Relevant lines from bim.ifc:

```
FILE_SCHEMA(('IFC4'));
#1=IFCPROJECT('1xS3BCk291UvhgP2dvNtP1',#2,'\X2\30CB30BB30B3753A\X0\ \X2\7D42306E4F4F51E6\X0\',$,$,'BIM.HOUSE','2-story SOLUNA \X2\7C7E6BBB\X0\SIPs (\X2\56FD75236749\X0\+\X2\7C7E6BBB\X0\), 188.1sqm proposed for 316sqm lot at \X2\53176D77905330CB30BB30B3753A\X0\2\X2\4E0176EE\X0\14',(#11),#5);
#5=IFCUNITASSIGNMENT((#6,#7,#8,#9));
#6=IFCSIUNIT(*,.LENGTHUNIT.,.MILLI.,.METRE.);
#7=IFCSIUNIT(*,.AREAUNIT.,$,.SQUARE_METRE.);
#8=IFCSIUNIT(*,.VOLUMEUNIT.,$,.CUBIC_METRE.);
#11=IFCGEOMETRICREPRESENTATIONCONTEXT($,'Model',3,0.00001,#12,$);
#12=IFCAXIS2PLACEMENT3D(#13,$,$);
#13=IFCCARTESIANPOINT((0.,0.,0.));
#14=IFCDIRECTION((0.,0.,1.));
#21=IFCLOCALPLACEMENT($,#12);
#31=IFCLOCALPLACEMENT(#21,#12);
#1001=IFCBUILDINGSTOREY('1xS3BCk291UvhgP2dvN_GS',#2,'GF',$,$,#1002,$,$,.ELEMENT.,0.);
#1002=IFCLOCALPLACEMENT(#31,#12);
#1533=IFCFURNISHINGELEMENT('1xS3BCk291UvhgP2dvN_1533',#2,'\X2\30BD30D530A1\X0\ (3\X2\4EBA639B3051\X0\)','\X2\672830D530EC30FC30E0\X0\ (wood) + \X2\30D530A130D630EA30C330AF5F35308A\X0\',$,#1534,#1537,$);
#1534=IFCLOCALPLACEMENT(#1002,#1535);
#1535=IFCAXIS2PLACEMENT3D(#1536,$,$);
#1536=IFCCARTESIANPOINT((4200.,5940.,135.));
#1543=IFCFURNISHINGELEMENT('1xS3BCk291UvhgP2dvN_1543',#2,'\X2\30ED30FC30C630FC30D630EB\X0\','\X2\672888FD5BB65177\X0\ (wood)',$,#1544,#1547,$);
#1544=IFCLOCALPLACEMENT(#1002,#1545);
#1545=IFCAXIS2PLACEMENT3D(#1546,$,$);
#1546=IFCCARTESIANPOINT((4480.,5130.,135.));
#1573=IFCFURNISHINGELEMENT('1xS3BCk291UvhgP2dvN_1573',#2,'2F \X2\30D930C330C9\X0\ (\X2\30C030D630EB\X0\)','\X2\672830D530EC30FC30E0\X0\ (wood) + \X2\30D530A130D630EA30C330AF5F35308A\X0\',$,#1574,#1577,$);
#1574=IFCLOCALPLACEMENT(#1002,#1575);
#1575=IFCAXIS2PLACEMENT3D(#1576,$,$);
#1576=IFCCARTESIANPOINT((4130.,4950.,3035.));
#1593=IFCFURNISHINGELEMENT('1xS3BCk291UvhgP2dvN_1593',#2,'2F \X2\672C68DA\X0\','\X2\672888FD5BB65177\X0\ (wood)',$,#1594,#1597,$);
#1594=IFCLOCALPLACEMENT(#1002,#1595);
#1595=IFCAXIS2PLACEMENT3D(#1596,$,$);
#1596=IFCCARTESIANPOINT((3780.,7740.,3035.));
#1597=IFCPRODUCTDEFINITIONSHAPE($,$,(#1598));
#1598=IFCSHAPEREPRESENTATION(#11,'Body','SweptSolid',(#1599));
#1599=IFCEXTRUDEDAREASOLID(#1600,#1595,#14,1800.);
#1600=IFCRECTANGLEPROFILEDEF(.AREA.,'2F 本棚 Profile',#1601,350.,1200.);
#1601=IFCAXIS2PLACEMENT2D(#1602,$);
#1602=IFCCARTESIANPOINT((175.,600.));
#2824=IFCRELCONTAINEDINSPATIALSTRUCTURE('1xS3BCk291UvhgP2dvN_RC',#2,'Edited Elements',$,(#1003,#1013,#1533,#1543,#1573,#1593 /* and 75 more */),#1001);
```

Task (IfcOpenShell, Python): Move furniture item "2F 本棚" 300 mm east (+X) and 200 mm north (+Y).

```python
import ifcopenshell
import ifcopenshell.api.geometry
import ifcopenshell.util.placement
import ifcopenshell.util.unit

model = ifcopenshell.open("bim.ifc")
unit_scale = ifcopenshell.util.unit.calculate_unit_scale(model)

item = model.by_guid("1xS3BCk291UvhgP2dvN_1593")
matrix = ifcopenshell.util.placement.get_local_placement(item.ObjectPlacement)
matrix[0, 3] += 0.3 / unit_scale
matrix[1, 3] += 0.2 / unit_scale
ifcopenshell.api.geometry.edit_object_placement(model, product=item, matrix=matrix, is_si=False)

print(ifcopenshell.util.placement.get_local_placement(item.ObjectPlacement).round(3) + 0.0)

model.write("bim_v2.ifc")
```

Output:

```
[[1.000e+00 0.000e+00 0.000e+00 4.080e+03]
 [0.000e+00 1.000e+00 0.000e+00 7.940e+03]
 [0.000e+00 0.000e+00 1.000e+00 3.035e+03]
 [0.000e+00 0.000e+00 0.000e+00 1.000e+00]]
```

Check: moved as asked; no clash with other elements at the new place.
